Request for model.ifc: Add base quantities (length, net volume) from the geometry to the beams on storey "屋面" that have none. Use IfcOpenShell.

First a look at what the model holds.

```python
import ifcopenshell
import ifcopenshell.util.element
import ifcopenshell.util.unit

model = ifcopenshell.open("model.ifc")
print(model.schema)
for unit_type in ("LENGTHUNIT", "AREAUNIT", "VOLUMEUNIT"):
    print(unit_type, ifcopenshell.util.unit.calculate_unit_scale(model, unit_type))
storey = next(s for s in model.by_type("IfcBuildingStorey") if s.Name == "屋面")
beams = [e for e in ifcopenshell.util.element.get_decomposition(storey) if e.is_a("IfcBeam")]
for e in sorted(beams, key=lambda e: e.id()):
    print(e.id(), e.is_a(), e.Name, list(ifcopenshell.util.element.get_psets(e, qtos_only=True)), sep=" | ")
```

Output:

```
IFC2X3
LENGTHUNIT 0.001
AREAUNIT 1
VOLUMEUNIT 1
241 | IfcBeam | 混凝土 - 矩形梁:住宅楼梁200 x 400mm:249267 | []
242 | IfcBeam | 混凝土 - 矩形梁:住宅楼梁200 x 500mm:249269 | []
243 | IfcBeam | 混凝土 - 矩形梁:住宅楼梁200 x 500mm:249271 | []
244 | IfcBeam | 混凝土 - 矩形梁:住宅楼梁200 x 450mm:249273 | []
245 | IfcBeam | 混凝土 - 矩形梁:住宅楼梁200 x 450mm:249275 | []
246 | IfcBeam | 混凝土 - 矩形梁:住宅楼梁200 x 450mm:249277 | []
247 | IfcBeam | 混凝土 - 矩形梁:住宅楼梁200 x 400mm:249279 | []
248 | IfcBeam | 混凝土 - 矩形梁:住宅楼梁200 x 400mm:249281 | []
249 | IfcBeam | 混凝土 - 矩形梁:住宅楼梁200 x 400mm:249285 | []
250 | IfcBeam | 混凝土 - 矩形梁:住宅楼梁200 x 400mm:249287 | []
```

```python
import ifcopenshell
import ifcopenshell.api.pset
import ifcopenshell.geom
import ifcopenshell.util.element
import ifcopenshell.util.shape
import ifcopenshell.util.unit

model = ifcopenshell.open("model.ifc")
unit_scale = ifcopenshell.util.unit.calculate_unit_scale(model)
volume_scale = ifcopenshell.util.unit.calculate_unit_scale(model, "VOLUMEUNIT")
settings = ifcopenshell.geom.settings()

storey = next(s for s in model.by_type("IfcBuildingStorey") if s.Name == "屋面")
beams = [e for e in ifcopenshell.util.element.get_decomposition(storey) if e.is_a("IfcBeam")]

for e in sorted(beams, key=lambda e: e.id()):
    if ifcopenshell.util.element.get_psets(e, qtos_only=True, should_inherit=False):
        continue
    # Geometry comes back in metres, in the element's own axes.
    shape = ifcopenshell.geom.create_shape(settings, e)
    values = {
        "Length": ifcopenshell.util.shape.get_max_xyz(shape.geometry) / unit_scale,
        "NetVolume": ifcopenshell.util.shape.get_volume(shape.geometry) / volume_scale,
    }
    qto = ifcopenshell.api.pset.add_qto(model, product=e, name="BaseQuantities")
    ifcopenshell.api.pset.edit_qto(model, qto=qto, properties=values)
    print(e.id(), {k: round(v, 3) for k, v in values.items()})

model.write("model_v2.ifc")
```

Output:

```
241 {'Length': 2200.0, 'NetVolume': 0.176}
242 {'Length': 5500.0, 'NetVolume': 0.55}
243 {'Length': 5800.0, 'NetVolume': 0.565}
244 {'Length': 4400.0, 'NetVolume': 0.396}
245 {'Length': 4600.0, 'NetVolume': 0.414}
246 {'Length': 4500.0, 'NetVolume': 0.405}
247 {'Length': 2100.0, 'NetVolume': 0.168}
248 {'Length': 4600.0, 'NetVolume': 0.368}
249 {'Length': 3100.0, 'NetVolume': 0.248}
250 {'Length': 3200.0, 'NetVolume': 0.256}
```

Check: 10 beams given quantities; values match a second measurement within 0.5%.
